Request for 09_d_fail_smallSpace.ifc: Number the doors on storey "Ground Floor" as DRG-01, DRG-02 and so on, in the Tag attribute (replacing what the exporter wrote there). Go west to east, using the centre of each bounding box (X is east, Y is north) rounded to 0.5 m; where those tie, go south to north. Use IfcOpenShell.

First a look at what the model holds.

```python
import ifcopenshell
import ifcopenshell.util.element
import ifcopenshell.util.placement

model = ifcopenshell.open("09_d_fail_smallSpace.ifc")
print(model.schema)
storey = next(s for s in model.by_type("IfcBuildingStorey") if s.Name == "Ground Floor")
doors = [e for e in ifcopenshell.util.element.get_decomposition(storey) if e.is_a("IfcDoor")]
for e in sorted(doors, key=lambda e: e.id()):
    origin = ifcopenshell.util.placement.get_local_placement(e.ObjectPlacement)[:3, 3]
    print(e.id(), e.Tag, e.Name, origin.round(2) + 0.0, sep=" | ")
```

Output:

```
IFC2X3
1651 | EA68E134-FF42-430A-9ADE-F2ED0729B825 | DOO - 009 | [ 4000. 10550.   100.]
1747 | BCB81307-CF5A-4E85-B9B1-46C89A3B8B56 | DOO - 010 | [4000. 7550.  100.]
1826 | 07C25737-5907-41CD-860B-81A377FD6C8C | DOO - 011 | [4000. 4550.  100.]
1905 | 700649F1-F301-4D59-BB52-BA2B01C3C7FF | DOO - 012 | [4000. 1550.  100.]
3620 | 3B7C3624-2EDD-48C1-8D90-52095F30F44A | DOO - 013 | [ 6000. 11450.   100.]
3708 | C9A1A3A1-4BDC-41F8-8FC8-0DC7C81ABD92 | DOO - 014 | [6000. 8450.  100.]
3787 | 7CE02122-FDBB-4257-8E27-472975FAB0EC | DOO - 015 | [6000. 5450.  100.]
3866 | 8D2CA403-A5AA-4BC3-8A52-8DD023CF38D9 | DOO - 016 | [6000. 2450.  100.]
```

```python
import ifcopenshell
import ifcopenshell.geom
import ifcopenshell.util.element
import ifcopenshell.util.shape

model = ifcopenshell.open("09_d_fail_smallSpace.ifc")
settings = ifcopenshell.geom.settings()
settings.set("use-world-coords", True)


def centre(element):
    shape = ifcopenshell.geom.create_shape(settings, element)
    return ifcopenshell.util.shape.get_bbox_centroid(shape.geometry)


storey = next(s for s in model.by_type("IfcBuildingStorey") if s.Name == "Ground Floor")
doors = [e for e in ifcopenshell.util.element.get_decomposition(storey) if e.is_a("IfcDoor")]

# Insertion points can sit at a corner or the storey origin, so sort by the geometry (in metres).
centres = {e: centre(e) for e in doors}
doors.sort(key=lambda e: (round(centres[e][0] / 0.5), centres[e][1]))

for i, e in enumerate(doors, start=1):
    number = f"DRG-{i:02d}"
    e.Tag = number
    print(e.id(), number)

model.write("09_d_fail_smallSpace_rev.ifc")
```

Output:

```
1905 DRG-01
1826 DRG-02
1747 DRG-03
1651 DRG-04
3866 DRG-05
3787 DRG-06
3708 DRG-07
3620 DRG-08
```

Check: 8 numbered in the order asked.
